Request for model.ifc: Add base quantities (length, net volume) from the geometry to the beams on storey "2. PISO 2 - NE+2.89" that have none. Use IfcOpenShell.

First a look at what the model holds.

```python
import ifcopenshell
import ifcopenshell.util.element
import ifcopenshell.util.unit

model = ifcopenshell.open("model.ifc")
print(model.schema)
for unit_type in ("LENGTHUNIT", "AREAUNIT", "VOLUMEUNIT"):
    print(unit_type, ifcopenshell.util.unit.calculate_unit_scale(model, unit_type))
storey = next(s for s in model.by_type("IfcBuildingStorey") if s.Name == "2. PISO 2 - NE+2.89")
beams = [e for e in ifcopenshell.util.element.get_decomposition(storey) if e.is_a("IfcBeam")]
for e in sorted(beams, key=lambda e: e.id()):
    print(e.id(), e.is_a(), e.Name, list(ifcopenshell.util.element.get_psets(e, qtos_only=True)), sep=" | ")
```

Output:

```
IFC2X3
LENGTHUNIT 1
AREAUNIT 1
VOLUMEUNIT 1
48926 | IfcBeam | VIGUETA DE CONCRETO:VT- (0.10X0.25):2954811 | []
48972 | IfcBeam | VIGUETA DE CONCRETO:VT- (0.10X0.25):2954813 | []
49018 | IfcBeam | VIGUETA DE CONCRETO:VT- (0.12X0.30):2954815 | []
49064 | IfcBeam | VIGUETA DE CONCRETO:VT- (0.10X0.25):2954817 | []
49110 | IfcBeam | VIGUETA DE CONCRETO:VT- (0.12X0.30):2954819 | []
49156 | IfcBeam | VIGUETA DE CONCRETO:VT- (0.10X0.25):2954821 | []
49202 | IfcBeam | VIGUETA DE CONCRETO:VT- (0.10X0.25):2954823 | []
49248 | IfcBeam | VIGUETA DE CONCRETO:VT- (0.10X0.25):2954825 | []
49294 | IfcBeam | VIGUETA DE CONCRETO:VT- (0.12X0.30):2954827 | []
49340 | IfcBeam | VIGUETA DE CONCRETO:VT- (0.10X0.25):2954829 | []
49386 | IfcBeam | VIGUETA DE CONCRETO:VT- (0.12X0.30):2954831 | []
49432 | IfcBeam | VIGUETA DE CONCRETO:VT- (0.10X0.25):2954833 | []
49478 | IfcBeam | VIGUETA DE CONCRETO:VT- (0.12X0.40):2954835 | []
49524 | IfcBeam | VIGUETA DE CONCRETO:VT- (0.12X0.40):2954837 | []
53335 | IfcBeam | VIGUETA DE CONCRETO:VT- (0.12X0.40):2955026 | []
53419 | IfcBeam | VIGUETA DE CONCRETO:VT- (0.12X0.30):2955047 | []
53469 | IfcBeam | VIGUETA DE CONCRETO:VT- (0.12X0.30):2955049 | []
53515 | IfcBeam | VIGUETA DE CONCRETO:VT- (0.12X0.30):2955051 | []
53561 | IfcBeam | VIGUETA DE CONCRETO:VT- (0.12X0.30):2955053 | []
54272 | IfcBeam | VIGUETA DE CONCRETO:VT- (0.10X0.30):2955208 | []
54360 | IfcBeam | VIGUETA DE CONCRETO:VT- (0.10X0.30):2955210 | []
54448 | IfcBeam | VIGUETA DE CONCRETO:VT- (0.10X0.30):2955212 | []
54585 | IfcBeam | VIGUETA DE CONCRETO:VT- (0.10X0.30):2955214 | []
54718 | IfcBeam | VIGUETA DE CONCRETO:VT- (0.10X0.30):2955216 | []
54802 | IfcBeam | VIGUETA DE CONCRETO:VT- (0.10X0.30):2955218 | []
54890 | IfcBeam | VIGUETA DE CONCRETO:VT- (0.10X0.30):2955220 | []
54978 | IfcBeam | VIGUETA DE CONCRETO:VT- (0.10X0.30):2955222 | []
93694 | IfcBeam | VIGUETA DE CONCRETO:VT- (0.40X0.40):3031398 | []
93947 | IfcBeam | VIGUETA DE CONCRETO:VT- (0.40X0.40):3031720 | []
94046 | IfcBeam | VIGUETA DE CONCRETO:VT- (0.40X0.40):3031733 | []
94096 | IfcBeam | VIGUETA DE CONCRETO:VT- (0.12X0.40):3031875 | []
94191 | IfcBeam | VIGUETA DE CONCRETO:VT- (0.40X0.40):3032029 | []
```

```python
import ifcopenshell
import ifcopenshell.api.pset
import ifcopenshell.geom
import ifcopenshell.util.element
import ifcopenshell.util.shape
import ifcopenshell.util.unit

model = ifcopenshell.open("model.ifc")
unit_scale = ifcopenshell.util.unit.calculate_unit_scale(model)
volume_scale = ifcopenshell.util.unit.calculate_unit_scale(model, "VOLUMEUNIT")
settings = ifcopenshell.geom.settings()

storey = next(s for s in model.by_type("IfcBuildingStorey") if s.Name == "2. PISO 2 - NE+2.89")
beams = [e for e in ifcopenshell.util.element.get_decomposition(storey) if e.is_a("IfcBeam")]

for e in sorted(beams, key=lambda e: e.id()):
    if ifcopenshell.util.element.get_psets(e, qtos_only=True, should_inherit=False):
        continue
    # Geometry comes back in metres, in the element's own axes.
    shape = ifcopenshell.geom.create_shape(settings, e)
    values = {
        "Length": ifcopenshell.util.shape.get_max_xyz(shape.geometry) / unit_scale,
        "NetVolume": ifcopenshell.util.shape.get_volume(shape.geometry) / volume_scale,
    }
    qto = ifcopenshell.api.pset.add_qto(model, product=e, name="BaseQuantities")
    ifcopenshell.api.pset.edit_qto(model, qto=qto, properties=values)
    print(e.id(), {k: round(v, 3) for k, v in values.items()})

model.write("model_updated.ifc")
```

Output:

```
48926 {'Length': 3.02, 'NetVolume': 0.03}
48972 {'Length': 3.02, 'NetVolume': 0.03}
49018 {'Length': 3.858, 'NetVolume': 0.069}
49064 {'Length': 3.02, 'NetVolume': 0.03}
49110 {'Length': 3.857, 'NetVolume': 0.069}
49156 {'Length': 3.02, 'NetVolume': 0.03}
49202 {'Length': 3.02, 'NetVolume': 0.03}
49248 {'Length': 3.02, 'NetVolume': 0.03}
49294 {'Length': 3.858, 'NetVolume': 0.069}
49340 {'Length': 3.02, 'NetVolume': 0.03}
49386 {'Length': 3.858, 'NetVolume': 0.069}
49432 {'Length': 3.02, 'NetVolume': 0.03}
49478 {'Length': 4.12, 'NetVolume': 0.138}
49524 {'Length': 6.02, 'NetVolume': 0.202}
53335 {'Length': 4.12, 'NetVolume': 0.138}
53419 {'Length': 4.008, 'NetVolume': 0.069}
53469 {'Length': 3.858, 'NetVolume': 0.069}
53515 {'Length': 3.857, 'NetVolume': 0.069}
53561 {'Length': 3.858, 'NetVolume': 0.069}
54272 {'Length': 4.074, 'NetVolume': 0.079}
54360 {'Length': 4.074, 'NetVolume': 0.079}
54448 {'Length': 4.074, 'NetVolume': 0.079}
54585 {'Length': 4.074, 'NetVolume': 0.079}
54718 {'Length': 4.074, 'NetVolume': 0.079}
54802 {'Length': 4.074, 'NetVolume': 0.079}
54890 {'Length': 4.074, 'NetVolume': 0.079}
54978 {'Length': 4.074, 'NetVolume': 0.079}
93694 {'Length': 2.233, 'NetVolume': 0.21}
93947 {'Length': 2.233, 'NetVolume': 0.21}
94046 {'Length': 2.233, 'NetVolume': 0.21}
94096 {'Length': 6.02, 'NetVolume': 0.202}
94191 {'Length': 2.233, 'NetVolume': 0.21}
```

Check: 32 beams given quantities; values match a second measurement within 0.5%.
